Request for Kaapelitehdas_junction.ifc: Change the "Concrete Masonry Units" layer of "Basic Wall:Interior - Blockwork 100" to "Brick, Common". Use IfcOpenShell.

First a look at what the model holds.

```python
import ifcopenshell
import ifcopenshell.util.element

model = ifcopenshell.open("Kaapelitehdas_junction.ifc")
print(model.schema)
for layer_set in model.by_type("IfcMaterialLayerSet"):
    if layer_set.LayerSetName == "Basic Wall:Interior - Blockwork 100":
        for layer in layer_set.MaterialLayers:
            print(layer.id(), layer.Material and layer.Material.Name, layer.LayerThickness, sep=" | ")
        print(len(ifcopenshell.util.element.get_elements_by_material(model, layer_set)), "elements and types use it")
print(sorted(m.Name for m in model.by_type("IfcMaterial") if m.Name)[:60])
```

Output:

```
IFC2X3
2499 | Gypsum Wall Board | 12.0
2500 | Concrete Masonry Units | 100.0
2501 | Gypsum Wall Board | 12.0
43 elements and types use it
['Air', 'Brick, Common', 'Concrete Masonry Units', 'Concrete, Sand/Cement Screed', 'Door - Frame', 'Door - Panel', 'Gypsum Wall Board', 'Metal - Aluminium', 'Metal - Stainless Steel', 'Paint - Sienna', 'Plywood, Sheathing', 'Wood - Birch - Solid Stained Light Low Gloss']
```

```python
import ifcopenshell
import ifcopenshell.api.material

model = ifcopenshell.open("Kaapelitehdas_junction.ifc")

layer_set = next(s for s in model.by_type("IfcMaterialLayerSet") if s.LayerSetName == "Basic Wall:Interior - Blockwork 100")
layer = next(l for l in layer_set.MaterialLayers if l.Material and l.Material.Name == "Concrete Masonry Units")
material = next(m for m in model.by_type("IfcMaterial") if m.Name == "Brick, Common")

# Point this one layer at the other material; renaming the old one would change it everywhere.
ifcopenshell.api.material.edit_layer(model, layer=layer, attributes={}, material=material)

print([l.Material.Name if l.Material else None for l in layer_set.MaterialLayers])

model.write("Kaapelitehdas_junction_updated.ifc")
```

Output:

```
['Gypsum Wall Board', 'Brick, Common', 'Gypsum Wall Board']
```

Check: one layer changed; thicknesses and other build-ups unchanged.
